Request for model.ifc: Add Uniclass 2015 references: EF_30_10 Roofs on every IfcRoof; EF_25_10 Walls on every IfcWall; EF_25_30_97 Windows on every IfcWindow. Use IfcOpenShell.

First a look at what the model holds.

```python
import ifcopenshell

model = ifcopenshell.open("model.ifc")
print(model.schema)
print("classifications:", [c.Name for c in model.by_type("IfcClassification")])
for ifc_class in ("IfcDoor", "IfcRoof", "IfcStair", "IfcWall", "IfcWindow"):
    print(ifc_class, len(model.by_type(ifc_class)))
```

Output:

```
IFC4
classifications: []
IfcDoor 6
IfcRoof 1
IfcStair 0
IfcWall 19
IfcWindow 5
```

```python
import ifcopenshell
import ifcopenshell.api.classification

model = ifcopenshell.open("model.ifc")

system = ifcopenshell.api.classification.add_classification(model, classification="Uniclass 2015")

codes = {
    "IfcRoof": ("EF_30_10", "Roofs"),
    "IfcWall": ("EF_25_10", "Walls"),
    "IfcWindow": ("EF_25_30_97", "Windows"),
}
for ifc_class, (code, name) in codes.items():
    products = model.by_type(ifc_class)
    ifcopenshell.api.classification.add_reference(
        model, products=products, classification=system, identification=code, name=name
    )
    print(code, len(products))

model.write("model_updated.ifc")
```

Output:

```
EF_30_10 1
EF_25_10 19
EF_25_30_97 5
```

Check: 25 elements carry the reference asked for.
